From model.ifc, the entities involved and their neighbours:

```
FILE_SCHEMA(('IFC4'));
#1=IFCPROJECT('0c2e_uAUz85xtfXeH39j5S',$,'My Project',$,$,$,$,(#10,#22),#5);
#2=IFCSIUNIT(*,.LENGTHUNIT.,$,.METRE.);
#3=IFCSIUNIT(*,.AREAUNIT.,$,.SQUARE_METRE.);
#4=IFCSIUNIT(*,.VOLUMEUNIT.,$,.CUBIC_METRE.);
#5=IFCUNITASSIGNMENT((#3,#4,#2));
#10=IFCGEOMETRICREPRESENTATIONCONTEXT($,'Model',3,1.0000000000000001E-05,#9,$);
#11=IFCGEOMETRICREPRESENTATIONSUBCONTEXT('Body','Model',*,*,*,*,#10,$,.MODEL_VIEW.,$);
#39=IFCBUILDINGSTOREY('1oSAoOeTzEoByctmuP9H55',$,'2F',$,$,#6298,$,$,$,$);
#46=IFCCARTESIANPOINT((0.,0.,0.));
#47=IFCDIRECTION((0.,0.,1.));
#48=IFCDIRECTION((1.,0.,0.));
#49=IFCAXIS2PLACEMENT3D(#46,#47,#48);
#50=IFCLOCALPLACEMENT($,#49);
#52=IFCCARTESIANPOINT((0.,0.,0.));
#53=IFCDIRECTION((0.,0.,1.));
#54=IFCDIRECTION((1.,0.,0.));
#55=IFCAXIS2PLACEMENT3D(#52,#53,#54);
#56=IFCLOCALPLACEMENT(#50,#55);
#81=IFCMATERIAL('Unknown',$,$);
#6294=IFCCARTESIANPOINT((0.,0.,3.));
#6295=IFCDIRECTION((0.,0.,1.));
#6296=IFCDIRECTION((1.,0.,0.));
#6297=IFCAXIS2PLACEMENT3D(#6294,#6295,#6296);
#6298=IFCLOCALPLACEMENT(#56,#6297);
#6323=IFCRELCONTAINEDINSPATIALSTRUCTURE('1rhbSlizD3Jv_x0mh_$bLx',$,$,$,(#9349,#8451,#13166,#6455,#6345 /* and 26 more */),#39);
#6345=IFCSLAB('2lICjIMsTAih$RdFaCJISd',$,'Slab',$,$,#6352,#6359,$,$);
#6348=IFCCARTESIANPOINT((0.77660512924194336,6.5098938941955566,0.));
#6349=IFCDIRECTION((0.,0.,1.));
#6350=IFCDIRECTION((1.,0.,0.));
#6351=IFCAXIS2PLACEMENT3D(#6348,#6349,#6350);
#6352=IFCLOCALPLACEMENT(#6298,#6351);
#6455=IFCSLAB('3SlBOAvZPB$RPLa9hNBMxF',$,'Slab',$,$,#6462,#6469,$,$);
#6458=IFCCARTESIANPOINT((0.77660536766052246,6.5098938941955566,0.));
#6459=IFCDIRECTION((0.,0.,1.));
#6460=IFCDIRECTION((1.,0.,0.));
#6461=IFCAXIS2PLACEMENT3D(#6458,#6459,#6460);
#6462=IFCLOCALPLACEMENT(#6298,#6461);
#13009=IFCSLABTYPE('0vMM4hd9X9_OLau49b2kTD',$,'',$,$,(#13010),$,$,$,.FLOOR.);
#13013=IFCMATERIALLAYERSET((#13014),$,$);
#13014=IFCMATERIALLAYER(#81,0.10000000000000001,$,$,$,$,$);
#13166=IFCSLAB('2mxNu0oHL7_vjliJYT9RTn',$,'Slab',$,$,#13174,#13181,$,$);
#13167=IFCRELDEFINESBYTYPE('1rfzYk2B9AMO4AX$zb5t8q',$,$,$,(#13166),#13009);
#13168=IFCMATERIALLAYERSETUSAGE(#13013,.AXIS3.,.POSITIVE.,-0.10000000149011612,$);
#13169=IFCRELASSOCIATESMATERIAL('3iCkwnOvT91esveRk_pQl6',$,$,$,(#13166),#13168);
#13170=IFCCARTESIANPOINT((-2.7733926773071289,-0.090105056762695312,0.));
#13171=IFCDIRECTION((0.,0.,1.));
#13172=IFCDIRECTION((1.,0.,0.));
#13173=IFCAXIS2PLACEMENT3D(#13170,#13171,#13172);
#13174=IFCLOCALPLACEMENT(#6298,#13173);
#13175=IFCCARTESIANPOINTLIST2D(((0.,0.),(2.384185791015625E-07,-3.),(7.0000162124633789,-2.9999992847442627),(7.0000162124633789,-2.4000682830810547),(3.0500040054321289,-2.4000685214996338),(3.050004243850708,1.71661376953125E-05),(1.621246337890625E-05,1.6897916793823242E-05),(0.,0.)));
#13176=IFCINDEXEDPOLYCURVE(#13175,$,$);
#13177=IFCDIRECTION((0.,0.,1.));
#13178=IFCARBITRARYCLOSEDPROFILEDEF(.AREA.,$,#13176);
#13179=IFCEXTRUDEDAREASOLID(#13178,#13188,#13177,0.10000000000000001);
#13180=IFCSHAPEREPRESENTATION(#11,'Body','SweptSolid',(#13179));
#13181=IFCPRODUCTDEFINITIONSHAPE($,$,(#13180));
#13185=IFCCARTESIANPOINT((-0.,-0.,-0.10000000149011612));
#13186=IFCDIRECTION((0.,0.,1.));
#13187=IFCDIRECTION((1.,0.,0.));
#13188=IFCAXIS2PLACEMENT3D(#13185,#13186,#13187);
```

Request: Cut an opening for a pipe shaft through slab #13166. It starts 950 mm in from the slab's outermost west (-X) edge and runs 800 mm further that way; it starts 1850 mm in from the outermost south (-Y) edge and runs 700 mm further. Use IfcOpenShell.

```python
import numpy as np
import ifcopenshell
import ifcopenshell.api.feature
import ifcopenshell.api.geometry
import ifcopenshell.api.root
import ifcopenshell.geom
import ifcopenshell.util.placement
import ifcopenshell.util.representation
import ifcopenshell.util.shape
import ifcopenshell.util.unit

model = ifcopenshell.open("model.ifc")
unit_scale = ifcopenshell.util.unit.calculate_unit_scale(model)
settings = ifcopenshell.geom.settings()


def volume(element):
    """Net volume in cubic metres, openings subtracted."""
    shape = ifcopenshell.geom.create_shape(settings, element)
    return ifcopenshell.util.shape.get_volume(shape.geometry)


slab = model.by_guid("2mxNu0oHL7_vjliJYT9RTn")
before = volume(slab)

# Extent in the slab's own axes, in metres. The edges named are its -X and -Y sides.
slab_shape = ifcopenshell.geom.create_shape(settings, slab)
vertices = ifcopenshell.util.shape.get_vertices(slab_shape.geometry)
x_min, y_min, bottom = vertices.min(axis=0)
top = vertices[:, 2].max()

opening = ifcopenshell.api.root.create_entity(model, ifc_class="IfcOpeningElement", name="Pipe shaft opening", predefined_type="OPENING")
context = ifcopenshell.util.representation.get_context(model, "Model", "Body", "MODEL_VIEW")
width, depth = 0.8, 0.7
outline = [(0.0, 0.0), (width, 0.0), (width, depth), (0.0, depth), (0.0, 0.0)]
# Overshoot both faces by 50 mm so the cut is clean.
shape = ifcopenshell.api.geometry.add_slab_representation(
    model, context=context, depth=top - bottom + 0.1, polyline=outline
)
ifcopenshell.api.geometry.assign_representation(model, product=opening, representation=shape)

matrix = ifcopenshell.util.placement.get_local_placement(slab.ObjectPlacement)
matrix[:, 3] = matrix @ np.append(np.array([x_min + 0.95, y_min + 1.85, bottom - 0.05]) / unit_scale, 1.0)
ifcopenshell.api.geometry.edit_object_placement(model, product=opening, matrix=matrix, is_si=False)
ifcopenshell.api.feature.add_feature(model, feature=opening, element=slab)

after = volume(slab)

print(f"slab volume {before:.3f} -> {after:.3f} m3")

model.write("model_v2.ifc")
```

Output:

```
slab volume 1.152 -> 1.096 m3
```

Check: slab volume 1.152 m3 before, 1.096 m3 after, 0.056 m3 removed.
